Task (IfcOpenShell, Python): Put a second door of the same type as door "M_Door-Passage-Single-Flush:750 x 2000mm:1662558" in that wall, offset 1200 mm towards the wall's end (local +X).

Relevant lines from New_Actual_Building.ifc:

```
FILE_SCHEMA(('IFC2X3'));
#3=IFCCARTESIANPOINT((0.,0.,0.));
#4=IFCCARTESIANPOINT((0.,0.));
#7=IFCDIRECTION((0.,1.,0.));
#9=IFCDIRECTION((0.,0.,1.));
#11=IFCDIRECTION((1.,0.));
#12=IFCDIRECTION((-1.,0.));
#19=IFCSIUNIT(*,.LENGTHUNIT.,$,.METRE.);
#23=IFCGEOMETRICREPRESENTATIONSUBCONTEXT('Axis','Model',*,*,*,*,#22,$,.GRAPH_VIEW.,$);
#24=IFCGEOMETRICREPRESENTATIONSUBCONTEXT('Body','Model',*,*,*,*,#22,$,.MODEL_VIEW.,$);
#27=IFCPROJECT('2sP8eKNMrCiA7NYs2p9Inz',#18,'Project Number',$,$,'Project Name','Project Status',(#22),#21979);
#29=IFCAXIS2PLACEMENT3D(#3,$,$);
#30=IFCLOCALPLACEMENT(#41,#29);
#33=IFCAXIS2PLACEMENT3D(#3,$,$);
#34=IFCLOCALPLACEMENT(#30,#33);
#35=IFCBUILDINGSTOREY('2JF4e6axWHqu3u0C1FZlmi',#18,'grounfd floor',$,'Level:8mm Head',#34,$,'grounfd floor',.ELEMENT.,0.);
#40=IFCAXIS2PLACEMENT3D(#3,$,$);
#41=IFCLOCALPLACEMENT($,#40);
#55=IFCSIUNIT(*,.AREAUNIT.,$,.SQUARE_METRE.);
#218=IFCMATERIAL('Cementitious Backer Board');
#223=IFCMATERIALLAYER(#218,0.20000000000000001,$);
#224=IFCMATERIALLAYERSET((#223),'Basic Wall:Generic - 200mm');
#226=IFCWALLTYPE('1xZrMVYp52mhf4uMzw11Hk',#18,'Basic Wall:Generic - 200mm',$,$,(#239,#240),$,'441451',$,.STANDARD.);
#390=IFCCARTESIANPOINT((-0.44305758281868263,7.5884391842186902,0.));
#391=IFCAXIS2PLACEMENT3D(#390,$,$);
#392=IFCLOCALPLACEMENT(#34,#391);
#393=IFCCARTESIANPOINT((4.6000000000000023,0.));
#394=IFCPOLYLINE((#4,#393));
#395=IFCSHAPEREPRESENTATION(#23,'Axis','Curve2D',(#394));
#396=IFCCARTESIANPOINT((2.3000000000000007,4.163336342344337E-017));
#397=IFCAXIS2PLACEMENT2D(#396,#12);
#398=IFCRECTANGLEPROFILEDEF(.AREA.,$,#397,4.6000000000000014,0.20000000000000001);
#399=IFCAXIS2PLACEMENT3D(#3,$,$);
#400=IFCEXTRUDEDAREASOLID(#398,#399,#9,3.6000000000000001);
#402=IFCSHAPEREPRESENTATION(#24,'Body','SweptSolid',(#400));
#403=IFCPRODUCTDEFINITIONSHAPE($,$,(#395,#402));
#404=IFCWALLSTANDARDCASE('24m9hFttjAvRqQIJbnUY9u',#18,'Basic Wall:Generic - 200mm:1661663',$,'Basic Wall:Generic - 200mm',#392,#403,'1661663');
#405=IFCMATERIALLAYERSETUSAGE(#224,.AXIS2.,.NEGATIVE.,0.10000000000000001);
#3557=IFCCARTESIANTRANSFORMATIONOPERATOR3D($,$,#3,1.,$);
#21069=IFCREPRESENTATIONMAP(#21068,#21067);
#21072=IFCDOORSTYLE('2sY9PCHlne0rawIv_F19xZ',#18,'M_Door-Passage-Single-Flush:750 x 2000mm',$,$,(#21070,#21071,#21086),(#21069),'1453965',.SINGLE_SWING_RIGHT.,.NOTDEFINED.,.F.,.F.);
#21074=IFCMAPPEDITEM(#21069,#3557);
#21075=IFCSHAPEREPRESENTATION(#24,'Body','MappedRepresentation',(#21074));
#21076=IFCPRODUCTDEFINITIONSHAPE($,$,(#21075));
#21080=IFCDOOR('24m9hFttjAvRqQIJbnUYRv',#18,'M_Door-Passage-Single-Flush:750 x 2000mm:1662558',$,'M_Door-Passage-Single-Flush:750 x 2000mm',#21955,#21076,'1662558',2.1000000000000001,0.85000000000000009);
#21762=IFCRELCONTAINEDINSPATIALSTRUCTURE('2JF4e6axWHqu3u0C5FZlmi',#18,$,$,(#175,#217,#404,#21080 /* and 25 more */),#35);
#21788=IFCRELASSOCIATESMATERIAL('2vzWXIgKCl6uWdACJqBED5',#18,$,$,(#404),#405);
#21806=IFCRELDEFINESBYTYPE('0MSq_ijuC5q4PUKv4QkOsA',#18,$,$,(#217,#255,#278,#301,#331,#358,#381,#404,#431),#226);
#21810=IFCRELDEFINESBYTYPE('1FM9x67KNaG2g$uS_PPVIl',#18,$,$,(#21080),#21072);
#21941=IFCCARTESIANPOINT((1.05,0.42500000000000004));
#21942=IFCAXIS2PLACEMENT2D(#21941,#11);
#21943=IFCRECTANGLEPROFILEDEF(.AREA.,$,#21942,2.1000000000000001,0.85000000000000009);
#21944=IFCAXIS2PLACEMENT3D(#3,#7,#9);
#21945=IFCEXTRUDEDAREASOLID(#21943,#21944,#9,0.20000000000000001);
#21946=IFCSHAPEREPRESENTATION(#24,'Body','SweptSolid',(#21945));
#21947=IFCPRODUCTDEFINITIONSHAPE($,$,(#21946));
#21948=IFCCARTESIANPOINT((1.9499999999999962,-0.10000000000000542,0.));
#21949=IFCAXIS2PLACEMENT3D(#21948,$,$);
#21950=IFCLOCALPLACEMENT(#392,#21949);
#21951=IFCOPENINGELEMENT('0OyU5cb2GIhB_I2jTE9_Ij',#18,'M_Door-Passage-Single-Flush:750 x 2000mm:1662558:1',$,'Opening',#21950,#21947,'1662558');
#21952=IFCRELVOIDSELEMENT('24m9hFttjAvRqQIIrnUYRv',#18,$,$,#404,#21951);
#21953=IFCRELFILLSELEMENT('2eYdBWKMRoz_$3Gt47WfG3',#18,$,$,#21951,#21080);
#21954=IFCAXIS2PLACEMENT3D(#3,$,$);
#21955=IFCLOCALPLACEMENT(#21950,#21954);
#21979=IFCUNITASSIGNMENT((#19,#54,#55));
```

```python
import ifcopenshell
import ifcopenshell.api.feature
import ifcopenshell.api.geometry
import ifcopenshell.api.root
import ifcopenshell.geom
import ifcopenshell.util.element
import ifcopenshell.util.placement
import ifcopenshell.util.shape
import ifcopenshell.util.unit

model = ifcopenshell.open("New_Actual_Building.ifc")
unit_scale = ifcopenshell.util.unit.calculate_unit_scale(model)
settings = ifcopenshell.geom.settings()


def volume(element):
    """Net volume in cubic metres, openings subtracted."""
    shape = ifcopenshell.geom.create_shape(settings, element)
    return ifcopenshell.util.shape.get_volume(shape.geometry)


def reuse_history(source, copy):
    """copy_class also copies each property set's owner history, people and application; keep the originals."""
    for rel in copy.IsDefinedBy:
        if rel.is_a("IfcRelDefinesByProperties") and (history := rel.RelatingPropertyDefinition.OwnerHistory):
            rel.RelatingPropertyDefinition.OwnerHistory = source.OwnerHistory
            ifcopenshell.util.element.remove_deep2(model, history)


door = model.by_guid("24m9hFttjAvRqQIJbnUYRv")
opening = door.FillsVoids[0].RelatingOpeningElement
wall = opening.VoidsElements[0].RelatingBuildingElement
before = volume(wall)
shift = ifcopenshell.util.placement.get_local_placement(wall.ObjectPlacement)[:3, 0] * 1.2 / unit_scale

# copy_class copies the void relationship, type, container and properties, but no geometry.
new_opening = ifcopenshell.api.root.copy_class(model, product=opening)
new_opening.Representation = ifcopenshell.util.element.copy_deep(
    model, opening.Representation, exclude=["IfcGeometricRepresentationContext", "IfcRepresentationMap"]
)
new_opening.Name = "M_Door-Passage-Single-Flush:750 x 2000mm"
new_opening.Tag = None
new_door = ifcopenshell.api.root.copy_class(model, product=door)
new_door.Representation = ifcopenshell.util.element.copy_deep(
    model, door.Representation, exclude=["IfcGeometricRepresentationContext", "IfcRepresentationMap"]
)
new_door.Name = "M_Door-Passage-Single-Flush:750 x 2000mm"
new_door.Tag = None
reuse_history(door, new_door)
fills = ifcopenshell.api.feature.add_filling(model, opening=new_opening, element=new_door)
fills.OwnerHistory = new_door.OwnerHistory  # required in IFC2X3

for old, new in ((opening, new_opening), (door, new_door)):
    matrix = ifcopenshell.util.placement.get_local_placement(old.ObjectPlacement)
    matrix[:3, 3] += shift
    ifcopenshell.api.geometry.edit_object_placement(model, product=new, matrix=matrix, is_si=False)

after = volume(wall)

print(f"wall volume {before:.3f} -> {after:.3f} m3")

model.write("New_Actual_Building_edited.ifc")
```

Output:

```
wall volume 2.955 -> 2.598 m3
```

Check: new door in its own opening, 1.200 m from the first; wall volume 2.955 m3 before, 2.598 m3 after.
